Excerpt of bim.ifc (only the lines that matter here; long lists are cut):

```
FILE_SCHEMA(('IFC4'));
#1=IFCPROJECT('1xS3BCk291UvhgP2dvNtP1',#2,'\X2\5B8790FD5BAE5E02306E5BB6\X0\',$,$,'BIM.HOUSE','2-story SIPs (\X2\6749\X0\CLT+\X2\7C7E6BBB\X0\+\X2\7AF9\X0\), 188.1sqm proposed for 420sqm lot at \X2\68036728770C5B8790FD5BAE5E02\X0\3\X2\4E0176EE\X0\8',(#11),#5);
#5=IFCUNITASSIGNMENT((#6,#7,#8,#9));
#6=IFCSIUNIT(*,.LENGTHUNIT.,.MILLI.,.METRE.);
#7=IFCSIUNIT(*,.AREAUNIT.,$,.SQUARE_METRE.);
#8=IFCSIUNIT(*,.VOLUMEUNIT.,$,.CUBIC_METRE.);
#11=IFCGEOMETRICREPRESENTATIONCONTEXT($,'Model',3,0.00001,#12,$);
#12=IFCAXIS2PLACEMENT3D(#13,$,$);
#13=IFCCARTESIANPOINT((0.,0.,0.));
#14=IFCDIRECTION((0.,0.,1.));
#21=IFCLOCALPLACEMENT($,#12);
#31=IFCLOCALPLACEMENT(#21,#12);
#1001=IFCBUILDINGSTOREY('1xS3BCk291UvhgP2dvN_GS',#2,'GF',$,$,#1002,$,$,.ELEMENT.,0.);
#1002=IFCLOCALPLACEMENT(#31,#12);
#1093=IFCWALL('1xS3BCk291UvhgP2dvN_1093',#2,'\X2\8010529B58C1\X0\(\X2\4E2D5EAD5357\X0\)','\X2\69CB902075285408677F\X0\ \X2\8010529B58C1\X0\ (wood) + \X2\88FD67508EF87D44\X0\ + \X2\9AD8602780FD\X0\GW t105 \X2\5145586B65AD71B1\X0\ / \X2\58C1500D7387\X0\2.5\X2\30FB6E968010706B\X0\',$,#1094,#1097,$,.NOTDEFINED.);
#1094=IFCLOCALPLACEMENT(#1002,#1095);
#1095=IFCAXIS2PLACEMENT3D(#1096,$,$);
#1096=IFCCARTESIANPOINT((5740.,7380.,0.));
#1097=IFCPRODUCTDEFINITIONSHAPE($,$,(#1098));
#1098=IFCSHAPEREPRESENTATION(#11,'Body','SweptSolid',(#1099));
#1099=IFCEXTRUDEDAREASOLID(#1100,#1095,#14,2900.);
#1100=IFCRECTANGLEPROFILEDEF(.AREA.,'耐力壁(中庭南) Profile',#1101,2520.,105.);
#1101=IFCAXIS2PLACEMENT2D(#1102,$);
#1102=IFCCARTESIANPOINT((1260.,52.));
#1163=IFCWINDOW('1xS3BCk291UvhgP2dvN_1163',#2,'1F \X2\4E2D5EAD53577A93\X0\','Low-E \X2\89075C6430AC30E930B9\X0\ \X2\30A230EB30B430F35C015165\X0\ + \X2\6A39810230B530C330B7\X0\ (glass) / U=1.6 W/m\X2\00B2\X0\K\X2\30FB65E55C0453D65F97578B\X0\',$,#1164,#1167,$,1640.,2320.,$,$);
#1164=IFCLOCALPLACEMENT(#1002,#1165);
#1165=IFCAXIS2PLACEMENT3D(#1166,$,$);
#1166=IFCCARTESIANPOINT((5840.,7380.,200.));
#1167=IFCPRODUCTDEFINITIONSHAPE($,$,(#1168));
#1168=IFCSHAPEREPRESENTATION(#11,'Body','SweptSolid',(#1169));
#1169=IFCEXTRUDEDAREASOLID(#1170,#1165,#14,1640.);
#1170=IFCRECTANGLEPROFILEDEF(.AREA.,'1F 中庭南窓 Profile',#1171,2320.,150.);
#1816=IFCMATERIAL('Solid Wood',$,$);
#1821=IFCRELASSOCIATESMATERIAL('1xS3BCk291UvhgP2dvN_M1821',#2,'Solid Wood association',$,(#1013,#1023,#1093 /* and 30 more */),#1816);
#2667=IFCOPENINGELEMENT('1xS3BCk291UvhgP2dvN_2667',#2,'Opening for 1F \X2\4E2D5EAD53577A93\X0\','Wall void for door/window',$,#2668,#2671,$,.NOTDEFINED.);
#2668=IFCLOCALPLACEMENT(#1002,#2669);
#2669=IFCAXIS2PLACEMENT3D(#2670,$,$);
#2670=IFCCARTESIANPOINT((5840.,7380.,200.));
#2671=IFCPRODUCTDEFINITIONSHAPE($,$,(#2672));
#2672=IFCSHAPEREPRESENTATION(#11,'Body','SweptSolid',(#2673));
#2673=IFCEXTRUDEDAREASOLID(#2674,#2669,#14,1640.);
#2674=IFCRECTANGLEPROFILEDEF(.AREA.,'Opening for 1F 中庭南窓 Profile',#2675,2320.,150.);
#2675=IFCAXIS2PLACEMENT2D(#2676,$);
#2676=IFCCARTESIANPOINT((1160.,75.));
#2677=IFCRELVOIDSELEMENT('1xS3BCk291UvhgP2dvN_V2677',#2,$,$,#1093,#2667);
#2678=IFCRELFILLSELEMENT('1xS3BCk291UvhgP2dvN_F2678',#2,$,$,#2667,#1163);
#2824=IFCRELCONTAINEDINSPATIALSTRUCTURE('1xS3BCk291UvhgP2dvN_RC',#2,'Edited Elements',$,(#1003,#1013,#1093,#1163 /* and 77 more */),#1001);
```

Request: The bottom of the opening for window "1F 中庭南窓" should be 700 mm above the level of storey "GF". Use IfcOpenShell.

```python
import numpy as np
import ifcopenshell
import ifcopenshell.api.geometry
import ifcopenshell.geom
import ifcopenshell.util.element
import ifcopenshell.util.placement
import ifcopenshell.util.shape
import ifcopenshell.util.unit

model = ifcopenshell.open("bim.ifc")
unit_scale = ifcopenshell.util.unit.calculate_unit_scale(model)

window = model.by_guid("1xS3BCk291UvhgP2dvN_1163")
opening = window.FillsVoids[0].RelatingOpeningElement
storey = ifcopenshell.util.element.get_container(window, ifc_class="IfcBuildingStorey")
level = ifcopenshell.util.placement.get_local_placement(storey.ObjectPlacement)[2, 3]

# The opening's origin need not be at the sill, so measure its lowest point.
shape = ifcopenshell.geom.create_shape(ifcopenshell.geom.settings(), opening)
bottom = ifcopenshell.util.shape.get_shape_bottom_elevation(shape, shape.geometry) / unit_scale
dz = level + 0.7 / unit_scale - bottom

shift = np.array([0.0, 0.0, dz])
# The window is not placed relative to its opening, so move both.
for product in (opening, window):
    matrix = ifcopenshell.util.placement.get_local_placement(product.ObjectPlacement)
    matrix[:3, 3] += shift
    ifcopenshell.api.geometry.edit_object_placement(model, product=product, matrix=matrix, is_si=False)

print(f"moved by {dz * unit_scale:+.3f} m")

model.write("bim_edited.ifc")
```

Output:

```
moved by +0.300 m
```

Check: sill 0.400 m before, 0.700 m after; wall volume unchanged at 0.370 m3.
